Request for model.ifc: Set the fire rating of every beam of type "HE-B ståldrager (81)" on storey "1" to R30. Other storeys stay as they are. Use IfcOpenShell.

First a look at what the model holds.

```python
import ifcopenshell
import ifcopenshell.util.element

model = ifcopenshell.open("model.ifc")
print(model.schema)
storey = next(s for s in model.by_type("IfcBuildingStorey") if s.Name == "1")
beams = [e for e in ifcopenshell.util.element.get_decomposition(storey) if e.is_a("IfcBeam")]
seen = {}
for e in beams:
    element_type = ifcopenshell.util.element.get_type(e)
    key = (element_type.Name if element_type != e and element_type else None, ifcopenshell.util.element.get_pset(e, "Pset_BeamCommon", "FireRating"))
    seen[key] = seen.get(key, 0) + 1
for (name, value), count in sorted(seen.items(), key=str):
    print(count, "x", name, "|", value)
```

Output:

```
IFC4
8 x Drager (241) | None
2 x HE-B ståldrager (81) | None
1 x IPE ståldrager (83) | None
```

```python
import ifcopenshell
import ifcopenshell.api.pset
import ifcopenshell.util.element

model = ifcopenshell.open("model.ifc")

storey = next(s for s in model.by_type("IfcBuildingStorey") if s.Name == "1")
beams = [e for e in ifcopenshell.util.element.get_decomposition(storey) if e.is_a("IfcBeam")]

count = 0
for e in beams:
    element_type = ifcopenshell.util.element.get_type(e)
    if element_type in (None, e) or element_type.Name != "HE-B ståldrager (81)":
        continue
    # add_pset returns the element's existing set when there is one.
    pset = ifcopenshell.api.pset.add_pset(model, product=e, name="Pset_BeamCommon")
    ifcopenshell.api.pset.edit_pset(model, pset=pset, properties={"FireRating": "R30"})
    count += 1

print(count, "beams updated")

model.write("model_edited.ifc")
```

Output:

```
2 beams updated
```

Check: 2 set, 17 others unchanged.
